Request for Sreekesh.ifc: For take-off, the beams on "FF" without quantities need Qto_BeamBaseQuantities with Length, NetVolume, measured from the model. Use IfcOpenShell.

First a look at what the model holds.

```python
import ifcopenshell
import ifcopenshell.util.element
import ifcopenshell.util.unit

model = ifcopenshell.open("Sreekesh.ifc")
print(model.schema)
for unit_type in ("LENGTHUNIT", "AREAUNIT", "VOLUMEUNIT"):
    print(unit_type, ifcopenshell.util.unit.calculate_unit_scale(model, unit_type))
storey = next(s for s in model.by_type("IfcBuildingStorey") if s.Name == "FF")
beams = [e for e in ifcopenshell.util.element.get_decomposition(storey) if e.is_a("IfcBeam")]
for e in sorted(beams, key=lambda e: e.id()):
    print(e.id(), e.is_a(), e.Name, list(ifcopenshell.util.element.get_psets(e, qtos_only=True)), sep=" | ")
```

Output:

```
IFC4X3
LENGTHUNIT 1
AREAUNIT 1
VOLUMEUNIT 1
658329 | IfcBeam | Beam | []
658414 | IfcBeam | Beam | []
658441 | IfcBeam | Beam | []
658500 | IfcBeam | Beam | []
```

```python
import ifcopenshell
import ifcopenshell.api.pset
import ifcopenshell.geom
import ifcopenshell.util.element
import ifcopenshell.util.shape
import ifcopenshell.util.unit

model = ifcopenshell.open("Sreekesh.ifc")
unit_scale = ifcopenshell.util.unit.calculate_unit_scale(model)
volume_scale = ifcopenshell.util.unit.calculate_unit_scale(model, "VOLUMEUNIT")
settings = ifcopenshell.geom.settings()

storey = next(s for s in model.by_type("IfcBuildingStorey") if s.Name == "FF")
beams = [e for e in ifcopenshell.util.element.get_decomposition(storey) if e.is_a("IfcBeam")]

for e in sorted(beams, key=lambda e: e.id()):
    if ifcopenshell.util.element.get_psets(e, qtos_only=True, should_inherit=False):
        continue
    # Geometry comes back in metres, in the element's own axes.
    shape = ifcopenshell.geom.create_shape(settings, e)
    values = {
        "Length": ifcopenshell.util.shape.get_max_xyz(shape.geometry) / unit_scale,
        "NetVolume": ifcopenshell.util.shape.get_volume(shape.geometry) / volume_scale,
    }
    qto = ifcopenshell.api.pset.add_qto(model, product=e, name="Qto_BeamBaseQuantities")
    ifcopenshell.api.pset.edit_qto(model, qto=qto, properties=values)
    print(e.id(), {k: round(v, 3) for k, v in values.items()})

model.write("Sreekesh_v2.ifc")
```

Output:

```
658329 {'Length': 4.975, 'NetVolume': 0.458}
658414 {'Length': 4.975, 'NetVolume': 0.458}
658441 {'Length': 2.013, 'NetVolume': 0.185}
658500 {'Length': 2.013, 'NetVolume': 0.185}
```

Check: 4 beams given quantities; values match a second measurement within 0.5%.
